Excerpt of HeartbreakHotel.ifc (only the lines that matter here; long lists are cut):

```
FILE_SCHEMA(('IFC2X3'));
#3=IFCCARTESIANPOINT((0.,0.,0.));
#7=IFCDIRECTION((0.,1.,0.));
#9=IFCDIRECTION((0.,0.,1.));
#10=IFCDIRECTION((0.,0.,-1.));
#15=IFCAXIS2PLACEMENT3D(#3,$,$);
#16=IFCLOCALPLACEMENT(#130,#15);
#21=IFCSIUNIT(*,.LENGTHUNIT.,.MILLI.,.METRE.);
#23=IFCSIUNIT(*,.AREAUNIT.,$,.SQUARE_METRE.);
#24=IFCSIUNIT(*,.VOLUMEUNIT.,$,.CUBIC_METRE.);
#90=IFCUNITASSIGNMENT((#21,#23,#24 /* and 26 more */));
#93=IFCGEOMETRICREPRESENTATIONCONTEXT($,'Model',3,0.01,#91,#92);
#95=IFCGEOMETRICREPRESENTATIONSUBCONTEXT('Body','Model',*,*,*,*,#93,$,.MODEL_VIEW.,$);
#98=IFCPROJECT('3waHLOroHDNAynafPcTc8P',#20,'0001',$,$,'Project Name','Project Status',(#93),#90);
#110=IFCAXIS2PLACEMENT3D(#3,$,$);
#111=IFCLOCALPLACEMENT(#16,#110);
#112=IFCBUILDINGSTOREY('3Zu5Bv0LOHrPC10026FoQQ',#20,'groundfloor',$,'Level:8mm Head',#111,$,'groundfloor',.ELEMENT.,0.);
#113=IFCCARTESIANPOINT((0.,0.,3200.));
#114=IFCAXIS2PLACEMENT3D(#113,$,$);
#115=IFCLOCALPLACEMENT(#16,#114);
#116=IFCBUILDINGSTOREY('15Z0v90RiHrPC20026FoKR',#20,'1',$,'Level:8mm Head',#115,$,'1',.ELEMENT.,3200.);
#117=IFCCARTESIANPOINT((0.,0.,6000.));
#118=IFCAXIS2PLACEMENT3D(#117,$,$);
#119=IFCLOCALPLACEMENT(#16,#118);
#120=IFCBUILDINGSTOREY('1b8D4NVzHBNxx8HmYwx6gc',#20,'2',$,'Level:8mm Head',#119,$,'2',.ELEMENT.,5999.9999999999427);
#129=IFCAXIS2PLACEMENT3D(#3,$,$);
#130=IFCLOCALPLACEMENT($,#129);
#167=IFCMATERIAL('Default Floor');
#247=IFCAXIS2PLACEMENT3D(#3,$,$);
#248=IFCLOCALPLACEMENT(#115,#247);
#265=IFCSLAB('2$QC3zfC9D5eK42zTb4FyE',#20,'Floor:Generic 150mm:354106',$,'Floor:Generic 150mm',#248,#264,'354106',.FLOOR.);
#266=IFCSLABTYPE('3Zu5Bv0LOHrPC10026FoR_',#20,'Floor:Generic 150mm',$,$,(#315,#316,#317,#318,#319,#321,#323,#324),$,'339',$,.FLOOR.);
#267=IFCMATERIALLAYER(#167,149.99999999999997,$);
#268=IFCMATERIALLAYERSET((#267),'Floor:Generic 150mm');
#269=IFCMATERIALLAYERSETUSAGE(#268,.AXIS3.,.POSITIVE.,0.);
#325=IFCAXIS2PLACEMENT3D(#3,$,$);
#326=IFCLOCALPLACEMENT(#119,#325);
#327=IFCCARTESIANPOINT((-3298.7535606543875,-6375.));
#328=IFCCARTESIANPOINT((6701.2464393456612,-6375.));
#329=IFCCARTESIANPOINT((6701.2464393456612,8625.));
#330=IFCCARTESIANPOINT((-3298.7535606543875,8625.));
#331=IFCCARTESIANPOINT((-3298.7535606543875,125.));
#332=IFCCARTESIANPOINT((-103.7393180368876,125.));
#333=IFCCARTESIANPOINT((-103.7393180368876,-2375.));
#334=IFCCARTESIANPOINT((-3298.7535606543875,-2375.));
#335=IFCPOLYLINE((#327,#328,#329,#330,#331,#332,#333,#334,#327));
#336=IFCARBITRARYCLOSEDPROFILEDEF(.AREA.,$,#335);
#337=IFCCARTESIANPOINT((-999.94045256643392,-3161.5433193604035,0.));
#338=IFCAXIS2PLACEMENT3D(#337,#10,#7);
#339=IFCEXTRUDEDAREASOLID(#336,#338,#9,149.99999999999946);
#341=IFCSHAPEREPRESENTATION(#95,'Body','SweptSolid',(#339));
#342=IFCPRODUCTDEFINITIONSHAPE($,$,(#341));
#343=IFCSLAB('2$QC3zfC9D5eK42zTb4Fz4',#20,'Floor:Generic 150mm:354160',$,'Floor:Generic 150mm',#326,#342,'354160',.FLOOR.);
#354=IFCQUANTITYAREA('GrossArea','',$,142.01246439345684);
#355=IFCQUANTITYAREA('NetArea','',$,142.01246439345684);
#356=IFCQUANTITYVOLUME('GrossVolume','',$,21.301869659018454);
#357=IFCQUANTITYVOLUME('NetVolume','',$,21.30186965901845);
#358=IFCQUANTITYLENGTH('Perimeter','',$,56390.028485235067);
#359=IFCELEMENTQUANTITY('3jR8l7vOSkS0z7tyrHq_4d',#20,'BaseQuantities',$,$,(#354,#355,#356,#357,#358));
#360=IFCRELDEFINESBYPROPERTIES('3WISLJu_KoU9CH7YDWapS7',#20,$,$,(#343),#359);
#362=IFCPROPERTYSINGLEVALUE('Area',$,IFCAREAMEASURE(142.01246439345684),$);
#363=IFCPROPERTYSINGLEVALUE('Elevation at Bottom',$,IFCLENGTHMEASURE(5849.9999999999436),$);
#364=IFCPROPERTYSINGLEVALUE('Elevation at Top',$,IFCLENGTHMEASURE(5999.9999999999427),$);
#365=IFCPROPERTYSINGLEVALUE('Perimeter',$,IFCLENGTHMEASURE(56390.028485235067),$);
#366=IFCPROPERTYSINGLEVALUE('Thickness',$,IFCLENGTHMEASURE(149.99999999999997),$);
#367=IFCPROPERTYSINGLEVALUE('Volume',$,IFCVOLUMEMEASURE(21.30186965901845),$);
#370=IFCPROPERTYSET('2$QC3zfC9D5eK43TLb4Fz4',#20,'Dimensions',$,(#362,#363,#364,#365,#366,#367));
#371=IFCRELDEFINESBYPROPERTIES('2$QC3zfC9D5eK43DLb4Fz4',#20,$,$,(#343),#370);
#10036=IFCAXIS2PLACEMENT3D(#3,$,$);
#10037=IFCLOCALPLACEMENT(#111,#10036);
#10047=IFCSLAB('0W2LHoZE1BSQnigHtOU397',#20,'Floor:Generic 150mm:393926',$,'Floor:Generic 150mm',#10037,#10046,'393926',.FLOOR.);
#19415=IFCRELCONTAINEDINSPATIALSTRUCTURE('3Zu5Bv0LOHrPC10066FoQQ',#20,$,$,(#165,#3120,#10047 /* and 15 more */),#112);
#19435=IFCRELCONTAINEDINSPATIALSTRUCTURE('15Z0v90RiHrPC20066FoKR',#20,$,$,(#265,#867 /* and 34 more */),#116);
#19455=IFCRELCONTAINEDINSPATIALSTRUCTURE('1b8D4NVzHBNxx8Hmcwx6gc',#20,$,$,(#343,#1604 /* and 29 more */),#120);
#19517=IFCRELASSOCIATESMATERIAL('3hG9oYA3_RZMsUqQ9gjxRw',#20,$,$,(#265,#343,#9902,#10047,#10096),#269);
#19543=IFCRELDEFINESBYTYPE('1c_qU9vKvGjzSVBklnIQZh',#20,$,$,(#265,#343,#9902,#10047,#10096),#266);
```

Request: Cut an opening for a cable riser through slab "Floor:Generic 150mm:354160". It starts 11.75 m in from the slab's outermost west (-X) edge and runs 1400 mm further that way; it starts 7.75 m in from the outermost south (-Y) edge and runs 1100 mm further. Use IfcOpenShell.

```python
import numpy as np
import ifcopenshell
import ifcopenshell.api.feature
import ifcopenshell.api.geometry
import ifcopenshell.api.pset
import ifcopenshell.api.root
import ifcopenshell.geom
import ifcopenshell.util.element
import ifcopenshell.util.placement
import ifcopenshell.util.representation
import ifcopenshell.util.shape
import ifcopenshell.util.unit

model = ifcopenshell.open("HeartbreakHotel.ifc")
unit_scale = ifcopenshell.util.unit.calculate_unit_scale(model)
area_scale = ifcopenshell.util.unit.calculate_unit_scale(model, "AREAUNIT")
volume_scale = ifcopenshell.util.unit.calculate_unit_scale(model, "VOLUMEUNIT")
settings = ifcopenshell.geom.settings()


def volume(element):
    """Net volume in cubic metres, openings subtracted."""
    shape = ifcopenshell.geom.create_shape(settings, element)
    return ifcopenshell.util.shape.get_volume(shape.geometry)


slab = model.by_guid("2$QC3zfC9D5eK42zTb4Fz4")
before = volume(slab)

# Extent in the slab's own axes, in metres. The edges named are its -X and -Y sides.
slab_shape = ifcopenshell.geom.create_shape(settings, slab)
vertices = ifcopenshell.util.shape.get_vertices(slab_shape.geometry)
x_min, y_min, bottom = vertices.min(axis=0)
top = vertices[:, 2].max()

opening = ifcopenshell.api.root.create_entity(model, ifc_class="IfcOpeningElement", name="Cable riser opening")
context = ifcopenshell.util.representation.get_context(model, "Model", "Body", "MODEL_VIEW")
width, depth = 1.4, 1.1
outline = [(0.0, 0.0), (width, 0.0), (width, depth), (0.0, depth), (0.0, 0.0)]
# Overshoot both faces by 50 mm so the cut is clean.
shape = ifcopenshell.api.geometry.add_slab_representation(
    model, context=context, depth=top - bottom + 0.1, polyline=outline
)
ifcopenshell.api.geometry.assign_representation(model, product=opening, representation=shape)

matrix = ifcopenshell.util.placement.get_local_placement(slab.ObjectPlacement)
matrix[:, 3] = matrix @ np.append(np.array([x_min + 11.75, y_min + 7.75, bottom - 0.05]) / unit_scale, 1.0)
ifcopenshell.api.geometry.edit_object_placement(model, product=opening, matrix=matrix, is_si=False)
ifcopenshell.api.feature.add_feature(model, feature=opening, element=slab)

after = volume(slab)

# Update the slab's stored quantities.
qto = model.by_id(ifcopenshell.util.element.get_pset(slab, "BaseQuantities", should_inherit=False)["id"])
ifcopenshell.api.pset.edit_qto(model, qto=qto, properties={
    "NetArea": after / (top - bottom) / area_scale,
    "NetVolume": after / volume_scale,
})
pset = model.by_id(ifcopenshell.util.element.get_pset(slab, "Dimensions", should_inherit=False)["id"])
ifcopenshell.api.pset.edit_pset(model, pset=pset, properties={
    "Area": model.create_entity("IfcAreaMeasure", after / (top - bottom) / area_scale),
    "Volume": model.create_entity("IfcVolumeMeasure", after / volume_scale),
})

print(f"slab volume {before:.3f} -> {after:.3f} m3")

model.write("HeartbreakHotel_updated.ifc")
```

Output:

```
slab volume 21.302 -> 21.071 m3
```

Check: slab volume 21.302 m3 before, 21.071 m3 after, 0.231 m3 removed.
